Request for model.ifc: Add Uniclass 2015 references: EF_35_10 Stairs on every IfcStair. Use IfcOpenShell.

First a look at what the model holds.

```python
import ifcopenshell

model = ifcopenshell.open("model.ifc")
print(model.schema)
print("classifications:", [c.Name for c in model.by_type("IfcClassification")])
for ifc_class in ("IfcDoor", "IfcRoof", "IfcStair", "IfcWall", "IfcWindow"):
    print(ifc_class, len(model.by_type(ifc_class)))
```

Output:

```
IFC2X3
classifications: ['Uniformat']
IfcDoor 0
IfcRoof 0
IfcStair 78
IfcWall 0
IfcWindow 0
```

```python
import ifcopenshell
import ifcopenshell.api.classification

model = ifcopenshell.open("model.ifc")

# IFC2X3 requires Source and Edition and has no link from the project to the system.
system = model.create_entity("IfcClassification", Source="NBS", Edition="2015", Name="Uniclass 2015")

codes = {
    "IfcStair": ("EF_35_10", "Stairs"),
}
for ifc_class, (code, name) in codes.items():
    products = model.by_type(ifc_class)
    ifcopenshell.api.classification.add_reference(
        model, products=products, classification=system, identification=code, name=name
    )
    print(code, len(products))

model.write("model_v2.ifc")
```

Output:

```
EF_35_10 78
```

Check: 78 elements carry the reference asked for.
